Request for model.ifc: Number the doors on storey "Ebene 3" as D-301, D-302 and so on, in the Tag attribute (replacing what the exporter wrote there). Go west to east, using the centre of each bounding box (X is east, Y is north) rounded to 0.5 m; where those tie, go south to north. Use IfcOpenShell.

First a look at what the model holds.

```python
import ifcopenshell
import ifcopenshell.util.element
import ifcopenshell.util.placement

model = ifcopenshell.open("model.ifc")
print(model.schema)
storey = next(s for s in model.by_type("IfcBuildingStorey") if s.Name == "Ebene 3")
doors = [e for e in ifcopenshell.util.element.get_decomposition(storey) if e.is_a("IfcDoor")]
for e in sorted(doors, key=lambda e: e.id()):
    origin = ifcopenshell.util.placement.get_local_placement(e.ObjectPlacement)[:3, 3]
    print(e.id(), e.Tag, e.Name, origin.round(2) + 0.0, sep=" | ")
```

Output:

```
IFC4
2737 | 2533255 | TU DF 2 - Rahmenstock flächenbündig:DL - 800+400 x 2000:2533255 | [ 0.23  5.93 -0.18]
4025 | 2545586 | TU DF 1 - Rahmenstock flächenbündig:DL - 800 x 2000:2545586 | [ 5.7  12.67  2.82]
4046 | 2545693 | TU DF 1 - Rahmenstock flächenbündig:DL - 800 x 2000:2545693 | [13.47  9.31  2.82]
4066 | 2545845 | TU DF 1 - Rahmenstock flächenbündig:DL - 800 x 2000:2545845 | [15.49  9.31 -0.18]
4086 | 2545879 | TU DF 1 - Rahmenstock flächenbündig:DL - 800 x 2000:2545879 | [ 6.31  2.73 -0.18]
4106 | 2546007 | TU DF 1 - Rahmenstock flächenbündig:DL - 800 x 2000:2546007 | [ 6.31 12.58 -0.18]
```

```python
import ifcopenshell
import ifcopenshell.geom
import ifcopenshell.util.element
import ifcopenshell.util.shape

model = ifcopenshell.open("model.ifc")
settings = ifcopenshell.geom.settings()
settings.set("use-world-coords", True)


def centre(element):
    shape = ifcopenshell.geom.create_shape(settings, element)
    return ifcopenshell.util.shape.get_bbox_centroid(shape.geometry)


storey = next(s for s in model.by_type("IfcBuildingStorey") if s.Name == "Ebene 3")
doors = [e for e in ifcopenshell.util.element.get_decomposition(storey) if e.is_a("IfcDoor")]

# Insertion points can sit at a corner or the storey origin, so sort by the geometry (in metres).
centres = {e: centre(e) for e in doors}
doors.sort(key=lambda e: (round(centres[e][0] / 0.5), centres[e][1]))

for i, e in enumerate(doors, start=1):
    number = f"D-3{i:02d}"
    e.Tag = number
    print(e.id(), number)

model.write("model-out.ifc")
```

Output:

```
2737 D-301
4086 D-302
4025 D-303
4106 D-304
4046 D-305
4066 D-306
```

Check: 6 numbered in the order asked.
